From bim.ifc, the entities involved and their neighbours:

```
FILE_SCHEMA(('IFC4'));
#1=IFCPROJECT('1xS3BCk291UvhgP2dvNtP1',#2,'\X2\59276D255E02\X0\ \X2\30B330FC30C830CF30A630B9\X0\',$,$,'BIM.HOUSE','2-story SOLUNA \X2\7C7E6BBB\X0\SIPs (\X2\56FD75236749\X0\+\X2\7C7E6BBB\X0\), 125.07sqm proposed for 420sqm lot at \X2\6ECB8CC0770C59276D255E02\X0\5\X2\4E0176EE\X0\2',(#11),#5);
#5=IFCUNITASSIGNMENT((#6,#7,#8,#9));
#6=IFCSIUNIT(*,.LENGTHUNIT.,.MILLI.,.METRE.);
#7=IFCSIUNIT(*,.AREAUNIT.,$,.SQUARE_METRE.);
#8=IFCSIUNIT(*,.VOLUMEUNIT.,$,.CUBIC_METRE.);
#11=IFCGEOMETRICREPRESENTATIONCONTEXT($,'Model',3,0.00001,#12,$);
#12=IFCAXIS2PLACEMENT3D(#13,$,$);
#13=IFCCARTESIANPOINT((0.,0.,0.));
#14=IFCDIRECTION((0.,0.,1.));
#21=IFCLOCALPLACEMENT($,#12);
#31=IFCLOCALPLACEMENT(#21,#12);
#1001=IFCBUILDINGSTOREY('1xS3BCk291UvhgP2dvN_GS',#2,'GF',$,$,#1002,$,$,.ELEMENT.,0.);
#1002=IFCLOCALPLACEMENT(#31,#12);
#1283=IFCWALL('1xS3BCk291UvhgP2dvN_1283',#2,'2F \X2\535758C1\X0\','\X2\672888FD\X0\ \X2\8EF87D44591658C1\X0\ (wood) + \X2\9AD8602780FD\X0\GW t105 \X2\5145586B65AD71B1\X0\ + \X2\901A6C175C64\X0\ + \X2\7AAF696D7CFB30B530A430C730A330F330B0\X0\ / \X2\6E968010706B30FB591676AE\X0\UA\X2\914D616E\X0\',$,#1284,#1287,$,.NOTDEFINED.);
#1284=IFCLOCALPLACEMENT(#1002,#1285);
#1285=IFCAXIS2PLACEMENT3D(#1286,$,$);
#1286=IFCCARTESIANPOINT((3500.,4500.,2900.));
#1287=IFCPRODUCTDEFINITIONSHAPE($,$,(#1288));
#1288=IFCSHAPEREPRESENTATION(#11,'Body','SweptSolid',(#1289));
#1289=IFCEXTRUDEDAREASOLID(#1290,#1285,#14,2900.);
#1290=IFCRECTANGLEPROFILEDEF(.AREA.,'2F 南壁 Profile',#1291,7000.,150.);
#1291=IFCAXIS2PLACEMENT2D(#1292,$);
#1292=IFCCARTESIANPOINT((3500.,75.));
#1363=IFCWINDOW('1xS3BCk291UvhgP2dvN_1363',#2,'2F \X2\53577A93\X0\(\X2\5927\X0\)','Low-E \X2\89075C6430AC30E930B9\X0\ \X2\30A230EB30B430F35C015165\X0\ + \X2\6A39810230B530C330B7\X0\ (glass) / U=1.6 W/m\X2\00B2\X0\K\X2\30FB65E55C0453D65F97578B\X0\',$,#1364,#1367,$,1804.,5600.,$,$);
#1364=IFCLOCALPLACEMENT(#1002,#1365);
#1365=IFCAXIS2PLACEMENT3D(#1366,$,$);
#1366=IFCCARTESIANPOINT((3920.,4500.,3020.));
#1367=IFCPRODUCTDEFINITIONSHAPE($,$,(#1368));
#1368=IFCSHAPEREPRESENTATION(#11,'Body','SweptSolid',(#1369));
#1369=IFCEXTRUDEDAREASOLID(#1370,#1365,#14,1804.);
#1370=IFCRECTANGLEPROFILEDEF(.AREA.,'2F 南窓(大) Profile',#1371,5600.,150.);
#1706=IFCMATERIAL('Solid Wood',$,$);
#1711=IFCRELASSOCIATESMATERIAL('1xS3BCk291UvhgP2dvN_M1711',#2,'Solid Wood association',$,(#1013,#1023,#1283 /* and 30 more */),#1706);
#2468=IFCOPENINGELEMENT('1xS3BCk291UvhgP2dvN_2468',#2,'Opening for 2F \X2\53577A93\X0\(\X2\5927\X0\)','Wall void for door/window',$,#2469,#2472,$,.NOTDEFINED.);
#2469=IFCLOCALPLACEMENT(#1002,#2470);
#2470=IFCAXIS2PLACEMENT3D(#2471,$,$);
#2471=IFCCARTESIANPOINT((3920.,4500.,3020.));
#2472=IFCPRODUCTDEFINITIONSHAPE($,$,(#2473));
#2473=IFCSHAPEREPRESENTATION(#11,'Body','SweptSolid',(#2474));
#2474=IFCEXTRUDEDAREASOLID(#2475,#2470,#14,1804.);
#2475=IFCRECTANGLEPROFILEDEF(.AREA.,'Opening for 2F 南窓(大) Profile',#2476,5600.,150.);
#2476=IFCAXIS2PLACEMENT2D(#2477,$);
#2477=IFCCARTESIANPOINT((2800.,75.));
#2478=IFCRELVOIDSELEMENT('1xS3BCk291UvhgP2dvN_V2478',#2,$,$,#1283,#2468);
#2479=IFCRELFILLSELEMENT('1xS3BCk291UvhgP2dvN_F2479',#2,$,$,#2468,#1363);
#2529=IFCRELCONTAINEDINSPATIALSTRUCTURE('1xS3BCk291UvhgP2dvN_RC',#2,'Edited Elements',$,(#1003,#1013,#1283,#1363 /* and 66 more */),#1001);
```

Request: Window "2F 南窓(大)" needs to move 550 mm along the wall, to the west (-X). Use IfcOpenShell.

```python
import ifcopenshell
import ifcopenshell.api.geometry
import ifcopenshell.util.placement

model = ifcopenshell.open("bim.ifc")

window = model.by_guid("1xS3BCk291UvhgP2dvN_1363")
opening = window.FillsVoids[0].RelatingOpeningElement
wall = opening.VoidsElements[0].RelatingBuildingElement

wall_matrix = ifcopenshell.util.placement.get_local_placement(wall.ObjectPlacement)
shift = wall_matrix[:3, 0] * -550.0
before = ifcopenshell.util.placement.get_local_placement(window.ObjectPlacement)[:3, 3].copy()

# The window is not placed relative to its opening, so move both.
for product in (opening, window):
    matrix = ifcopenshell.util.placement.get_local_placement(product.ObjectPlacement)
    matrix[:3, 3] += shift
    ifcopenshell.api.geometry.edit_object_placement(model, product=product, matrix=matrix, is_si=False)

after = ifcopenshell.util.placement.get_local_placement(window.ObjectPlacement)[:3, 3]
print("window moved by", (after - before).round(3) + 0.0)

model.write("bim_updated.ifc")
```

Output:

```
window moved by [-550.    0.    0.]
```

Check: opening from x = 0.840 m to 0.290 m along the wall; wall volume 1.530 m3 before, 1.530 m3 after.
